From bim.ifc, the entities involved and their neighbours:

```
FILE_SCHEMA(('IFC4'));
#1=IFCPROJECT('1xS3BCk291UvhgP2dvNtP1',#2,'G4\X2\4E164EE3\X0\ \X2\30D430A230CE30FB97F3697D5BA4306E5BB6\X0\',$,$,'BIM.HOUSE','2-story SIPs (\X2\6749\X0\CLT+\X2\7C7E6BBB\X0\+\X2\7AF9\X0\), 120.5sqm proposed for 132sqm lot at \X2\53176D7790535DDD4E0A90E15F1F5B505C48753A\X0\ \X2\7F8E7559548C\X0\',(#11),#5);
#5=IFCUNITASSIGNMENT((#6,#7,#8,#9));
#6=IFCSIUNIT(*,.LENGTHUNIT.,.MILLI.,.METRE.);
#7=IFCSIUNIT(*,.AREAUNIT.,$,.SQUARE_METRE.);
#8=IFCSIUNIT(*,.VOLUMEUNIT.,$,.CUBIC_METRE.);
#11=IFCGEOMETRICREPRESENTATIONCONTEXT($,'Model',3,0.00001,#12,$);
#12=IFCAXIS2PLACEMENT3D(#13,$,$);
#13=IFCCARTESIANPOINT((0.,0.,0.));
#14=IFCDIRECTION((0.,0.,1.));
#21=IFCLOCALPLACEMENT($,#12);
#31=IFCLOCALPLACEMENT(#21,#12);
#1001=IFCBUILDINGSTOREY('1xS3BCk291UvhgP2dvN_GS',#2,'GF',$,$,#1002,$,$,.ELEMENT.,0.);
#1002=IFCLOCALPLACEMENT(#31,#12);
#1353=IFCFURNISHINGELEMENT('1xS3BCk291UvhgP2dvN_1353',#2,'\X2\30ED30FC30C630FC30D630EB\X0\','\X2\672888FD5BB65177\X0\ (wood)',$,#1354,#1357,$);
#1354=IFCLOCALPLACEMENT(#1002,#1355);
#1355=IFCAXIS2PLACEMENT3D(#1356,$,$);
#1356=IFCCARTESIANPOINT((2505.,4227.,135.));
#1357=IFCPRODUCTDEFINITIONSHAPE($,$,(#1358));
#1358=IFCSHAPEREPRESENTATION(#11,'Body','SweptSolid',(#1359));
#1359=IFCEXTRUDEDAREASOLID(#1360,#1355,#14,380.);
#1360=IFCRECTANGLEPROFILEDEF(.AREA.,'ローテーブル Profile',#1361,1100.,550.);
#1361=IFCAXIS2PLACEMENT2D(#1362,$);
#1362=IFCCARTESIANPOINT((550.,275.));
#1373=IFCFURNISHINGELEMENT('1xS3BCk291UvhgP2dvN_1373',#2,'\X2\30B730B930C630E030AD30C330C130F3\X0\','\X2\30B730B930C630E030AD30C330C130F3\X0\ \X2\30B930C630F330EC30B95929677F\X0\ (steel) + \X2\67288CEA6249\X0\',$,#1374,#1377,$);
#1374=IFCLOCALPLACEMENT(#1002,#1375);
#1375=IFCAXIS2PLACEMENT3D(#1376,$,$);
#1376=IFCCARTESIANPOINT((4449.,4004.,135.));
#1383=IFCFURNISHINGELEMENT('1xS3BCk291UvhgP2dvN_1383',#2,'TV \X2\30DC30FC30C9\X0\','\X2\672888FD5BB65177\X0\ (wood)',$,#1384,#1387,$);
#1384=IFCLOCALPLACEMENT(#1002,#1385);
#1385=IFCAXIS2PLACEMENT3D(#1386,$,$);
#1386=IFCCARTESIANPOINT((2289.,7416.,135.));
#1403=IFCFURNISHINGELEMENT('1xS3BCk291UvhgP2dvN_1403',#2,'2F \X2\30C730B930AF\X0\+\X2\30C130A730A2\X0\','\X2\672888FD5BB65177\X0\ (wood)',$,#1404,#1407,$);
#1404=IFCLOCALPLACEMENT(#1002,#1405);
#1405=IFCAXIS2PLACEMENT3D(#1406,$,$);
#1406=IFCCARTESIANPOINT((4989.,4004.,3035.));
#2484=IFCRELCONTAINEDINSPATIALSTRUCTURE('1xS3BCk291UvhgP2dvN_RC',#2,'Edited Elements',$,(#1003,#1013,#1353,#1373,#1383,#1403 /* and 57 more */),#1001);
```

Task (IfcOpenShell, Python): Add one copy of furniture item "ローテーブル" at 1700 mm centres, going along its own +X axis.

```python
import ifcopenshell
import ifcopenshell.api.geometry
import ifcopenshell.api.root
import ifcopenshell.util.element
import ifcopenshell.util.placement
import ifcopenshell.util.unit

model = ifcopenshell.open("bim.ifc")
unit_scale = ifcopenshell.util.unit.calculate_unit_scale(model)


def reuse_history(source, copy):
    """copy_class also copies each property set's owner history, people and application; keep the originals."""
    for rel in copy.IsDefinedBy:
        if rel.is_a("IfcRelDefinesByProperties") and (history := rel.RelatingPropertyDefinition.OwnerHistory):
            rel.RelatingPropertyDefinition.OwnerHistory = source.OwnerHistory
            ifcopenshell.util.element.remove_deep2(model, history)


source = model.by_id(1353)
base = ifcopenshell.util.placement.get_local_placement(source.ObjectPlacement)
step = base[:3, 0] * 1.7 / unit_scale

for i in range(1, 2):
    copy = ifcopenshell.api.root.copy_class(model, product=source)
    copy.Representation = ifcopenshell.util.element.copy_deep(
        model, source.Representation, exclude=["IfcGeometricRepresentationContext", "IfcRepresentationMap"]
    )
    reuse_history(source, copy)
    matrix = base.copy()
    matrix[:3, 3] += i * step
    print("added at", matrix[:3, 3].round(3) + 0.0)
    ifcopenshell.api.geometry.edit_object_placement(model, product=copy, matrix=matrix, is_si=False)

model.write("bim_edited.ifc")
```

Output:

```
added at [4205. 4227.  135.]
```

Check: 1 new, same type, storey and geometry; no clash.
